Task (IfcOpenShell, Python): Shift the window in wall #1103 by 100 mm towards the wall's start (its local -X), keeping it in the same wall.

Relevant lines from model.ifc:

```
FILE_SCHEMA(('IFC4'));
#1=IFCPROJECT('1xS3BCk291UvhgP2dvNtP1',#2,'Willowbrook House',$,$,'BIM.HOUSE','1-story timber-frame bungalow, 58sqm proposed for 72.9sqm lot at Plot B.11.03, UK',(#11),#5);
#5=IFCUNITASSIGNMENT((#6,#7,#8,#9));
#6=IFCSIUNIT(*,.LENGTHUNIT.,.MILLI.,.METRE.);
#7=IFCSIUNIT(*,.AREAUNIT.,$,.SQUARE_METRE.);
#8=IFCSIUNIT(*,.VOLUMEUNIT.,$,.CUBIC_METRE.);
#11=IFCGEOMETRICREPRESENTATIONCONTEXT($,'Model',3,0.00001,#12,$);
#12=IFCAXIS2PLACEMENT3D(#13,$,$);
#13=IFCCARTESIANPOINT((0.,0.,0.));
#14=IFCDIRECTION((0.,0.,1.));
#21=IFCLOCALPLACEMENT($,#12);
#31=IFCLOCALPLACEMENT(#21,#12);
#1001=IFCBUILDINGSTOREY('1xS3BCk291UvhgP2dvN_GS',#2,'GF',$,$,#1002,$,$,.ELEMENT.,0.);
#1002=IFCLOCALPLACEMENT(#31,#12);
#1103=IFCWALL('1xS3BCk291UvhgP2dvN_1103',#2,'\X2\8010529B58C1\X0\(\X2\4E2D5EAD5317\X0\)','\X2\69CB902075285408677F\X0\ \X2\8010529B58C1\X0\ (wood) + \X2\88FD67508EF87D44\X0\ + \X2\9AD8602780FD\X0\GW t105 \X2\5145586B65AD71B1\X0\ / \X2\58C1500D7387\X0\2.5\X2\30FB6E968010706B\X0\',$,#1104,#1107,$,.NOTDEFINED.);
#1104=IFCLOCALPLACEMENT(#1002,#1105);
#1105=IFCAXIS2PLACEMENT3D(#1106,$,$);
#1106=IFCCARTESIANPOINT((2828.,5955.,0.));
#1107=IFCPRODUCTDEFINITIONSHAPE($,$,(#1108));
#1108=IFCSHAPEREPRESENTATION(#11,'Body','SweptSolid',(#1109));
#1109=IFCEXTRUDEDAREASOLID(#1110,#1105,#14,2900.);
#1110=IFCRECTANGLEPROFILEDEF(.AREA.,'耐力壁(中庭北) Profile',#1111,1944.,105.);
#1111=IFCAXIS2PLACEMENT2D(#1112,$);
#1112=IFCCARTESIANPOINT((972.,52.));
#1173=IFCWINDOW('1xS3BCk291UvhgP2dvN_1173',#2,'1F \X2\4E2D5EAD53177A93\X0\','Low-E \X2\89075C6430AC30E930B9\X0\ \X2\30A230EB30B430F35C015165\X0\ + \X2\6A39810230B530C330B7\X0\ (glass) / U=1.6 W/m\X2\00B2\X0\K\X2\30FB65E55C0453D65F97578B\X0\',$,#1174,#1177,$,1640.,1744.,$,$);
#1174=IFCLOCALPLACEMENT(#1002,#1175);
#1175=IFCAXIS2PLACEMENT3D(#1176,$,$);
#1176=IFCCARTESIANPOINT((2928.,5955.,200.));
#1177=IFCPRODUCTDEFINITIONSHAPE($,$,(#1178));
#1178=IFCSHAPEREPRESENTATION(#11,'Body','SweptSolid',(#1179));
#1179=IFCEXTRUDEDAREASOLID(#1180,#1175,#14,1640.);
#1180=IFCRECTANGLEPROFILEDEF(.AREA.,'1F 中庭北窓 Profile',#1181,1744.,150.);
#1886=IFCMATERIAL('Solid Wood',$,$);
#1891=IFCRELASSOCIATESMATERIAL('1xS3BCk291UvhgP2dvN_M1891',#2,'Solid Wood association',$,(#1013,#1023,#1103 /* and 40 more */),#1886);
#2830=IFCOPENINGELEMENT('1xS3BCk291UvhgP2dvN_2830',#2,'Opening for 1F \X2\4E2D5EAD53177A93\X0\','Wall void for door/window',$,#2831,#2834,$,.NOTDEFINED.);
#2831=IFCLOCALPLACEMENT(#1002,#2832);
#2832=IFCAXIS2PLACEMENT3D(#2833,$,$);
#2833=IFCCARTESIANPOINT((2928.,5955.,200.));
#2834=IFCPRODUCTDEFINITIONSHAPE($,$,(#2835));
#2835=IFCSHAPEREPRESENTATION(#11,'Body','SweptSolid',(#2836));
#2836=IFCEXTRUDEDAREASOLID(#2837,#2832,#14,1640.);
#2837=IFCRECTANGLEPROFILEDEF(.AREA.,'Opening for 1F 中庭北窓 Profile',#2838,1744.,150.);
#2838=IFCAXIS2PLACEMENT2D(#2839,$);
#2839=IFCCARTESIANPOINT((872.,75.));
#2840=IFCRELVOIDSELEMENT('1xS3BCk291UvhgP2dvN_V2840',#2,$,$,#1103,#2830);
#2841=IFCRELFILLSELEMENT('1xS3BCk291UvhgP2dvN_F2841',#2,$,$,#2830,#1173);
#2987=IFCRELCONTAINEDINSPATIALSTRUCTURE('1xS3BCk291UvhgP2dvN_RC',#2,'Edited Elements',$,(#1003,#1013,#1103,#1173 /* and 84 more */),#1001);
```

```python
import ifcopenshell
import ifcopenshell.api.geometry
import ifcopenshell.util.placement
import ifcopenshell.util.unit

model = ifcopenshell.open("model.ifc")
unit_scale = ifcopenshell.util.unit.calculate_unit_scale(model)

window = model.by_guid("1xS3BCk291UvhgP2dvN_1173")
opening = window.FillsVoids[0].RelatingOpeningElement
wall = opening.VoidsElements[0].RelatingBuildingElement

wall_matrix = ifcopenshell.util.placement.get_local_placement(wall.ObjectPlacement)
shift = wall_matrix[:3, 0] * -0.1 / unit_scale
before = ifcopenshell.util.placement.get_local_placement(window.ObjectPlacement)[:3, 3].copy()

# The window is not placed relative to its opening, so move both.
for product in (opening, window):
    matrix = ifcopenshell.util.placement.get_local_placement(product.ObjectPlacement)
    matrix[:3, 3] += shift
    ifcopenshell.api.geometry.edit_object_placement(model, product=product, matrix=matrix, is_si=False)

after = ifcopenshell.util.placement.get_local_placement(window.ObjectPlacement)[:3, 3]
print("window moved by", (after - before).round(3) + 0.0)

model.write("model_edited.ifc")
```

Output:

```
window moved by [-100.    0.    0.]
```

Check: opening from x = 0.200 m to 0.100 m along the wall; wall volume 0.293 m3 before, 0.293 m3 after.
